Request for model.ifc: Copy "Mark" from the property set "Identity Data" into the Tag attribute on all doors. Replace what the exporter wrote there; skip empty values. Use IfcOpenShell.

First a look at what the model holds.

```python
import ifcopenshell
import ifcopenshell.util.element

model = ifcopenshell.open("model.ifc")
print(model.schema)
doors = model.by_type("IfcDoor")
print(len(doors), "doors")
for e in doors[:8]:
    source = ifcopenshell.util.element.get_pset(e, "Identity Data", "Mark")
    target = e.Tag
    print(e.id(), repr(source), repr(target), sep=" | ")
```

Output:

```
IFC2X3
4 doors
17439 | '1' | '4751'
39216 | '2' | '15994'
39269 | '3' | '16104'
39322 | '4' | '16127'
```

```python
import ifcopenshell
import ifcopenshell.util.element

model = ifcopenshell.open("model.ifc")

count = 0
for e in model.by_type("IfcDoor"):
    value = ifcopenshell.util.element.get_pset(e, "Identity Data", "Mark")
    current = e.Tag
    if not value or not value.strip() or current == value:
        continue
    e.Tag = value
    count += 1

print(count, "doors updated")

model.write("model_rev.ifc")
```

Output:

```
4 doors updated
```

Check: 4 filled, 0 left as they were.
